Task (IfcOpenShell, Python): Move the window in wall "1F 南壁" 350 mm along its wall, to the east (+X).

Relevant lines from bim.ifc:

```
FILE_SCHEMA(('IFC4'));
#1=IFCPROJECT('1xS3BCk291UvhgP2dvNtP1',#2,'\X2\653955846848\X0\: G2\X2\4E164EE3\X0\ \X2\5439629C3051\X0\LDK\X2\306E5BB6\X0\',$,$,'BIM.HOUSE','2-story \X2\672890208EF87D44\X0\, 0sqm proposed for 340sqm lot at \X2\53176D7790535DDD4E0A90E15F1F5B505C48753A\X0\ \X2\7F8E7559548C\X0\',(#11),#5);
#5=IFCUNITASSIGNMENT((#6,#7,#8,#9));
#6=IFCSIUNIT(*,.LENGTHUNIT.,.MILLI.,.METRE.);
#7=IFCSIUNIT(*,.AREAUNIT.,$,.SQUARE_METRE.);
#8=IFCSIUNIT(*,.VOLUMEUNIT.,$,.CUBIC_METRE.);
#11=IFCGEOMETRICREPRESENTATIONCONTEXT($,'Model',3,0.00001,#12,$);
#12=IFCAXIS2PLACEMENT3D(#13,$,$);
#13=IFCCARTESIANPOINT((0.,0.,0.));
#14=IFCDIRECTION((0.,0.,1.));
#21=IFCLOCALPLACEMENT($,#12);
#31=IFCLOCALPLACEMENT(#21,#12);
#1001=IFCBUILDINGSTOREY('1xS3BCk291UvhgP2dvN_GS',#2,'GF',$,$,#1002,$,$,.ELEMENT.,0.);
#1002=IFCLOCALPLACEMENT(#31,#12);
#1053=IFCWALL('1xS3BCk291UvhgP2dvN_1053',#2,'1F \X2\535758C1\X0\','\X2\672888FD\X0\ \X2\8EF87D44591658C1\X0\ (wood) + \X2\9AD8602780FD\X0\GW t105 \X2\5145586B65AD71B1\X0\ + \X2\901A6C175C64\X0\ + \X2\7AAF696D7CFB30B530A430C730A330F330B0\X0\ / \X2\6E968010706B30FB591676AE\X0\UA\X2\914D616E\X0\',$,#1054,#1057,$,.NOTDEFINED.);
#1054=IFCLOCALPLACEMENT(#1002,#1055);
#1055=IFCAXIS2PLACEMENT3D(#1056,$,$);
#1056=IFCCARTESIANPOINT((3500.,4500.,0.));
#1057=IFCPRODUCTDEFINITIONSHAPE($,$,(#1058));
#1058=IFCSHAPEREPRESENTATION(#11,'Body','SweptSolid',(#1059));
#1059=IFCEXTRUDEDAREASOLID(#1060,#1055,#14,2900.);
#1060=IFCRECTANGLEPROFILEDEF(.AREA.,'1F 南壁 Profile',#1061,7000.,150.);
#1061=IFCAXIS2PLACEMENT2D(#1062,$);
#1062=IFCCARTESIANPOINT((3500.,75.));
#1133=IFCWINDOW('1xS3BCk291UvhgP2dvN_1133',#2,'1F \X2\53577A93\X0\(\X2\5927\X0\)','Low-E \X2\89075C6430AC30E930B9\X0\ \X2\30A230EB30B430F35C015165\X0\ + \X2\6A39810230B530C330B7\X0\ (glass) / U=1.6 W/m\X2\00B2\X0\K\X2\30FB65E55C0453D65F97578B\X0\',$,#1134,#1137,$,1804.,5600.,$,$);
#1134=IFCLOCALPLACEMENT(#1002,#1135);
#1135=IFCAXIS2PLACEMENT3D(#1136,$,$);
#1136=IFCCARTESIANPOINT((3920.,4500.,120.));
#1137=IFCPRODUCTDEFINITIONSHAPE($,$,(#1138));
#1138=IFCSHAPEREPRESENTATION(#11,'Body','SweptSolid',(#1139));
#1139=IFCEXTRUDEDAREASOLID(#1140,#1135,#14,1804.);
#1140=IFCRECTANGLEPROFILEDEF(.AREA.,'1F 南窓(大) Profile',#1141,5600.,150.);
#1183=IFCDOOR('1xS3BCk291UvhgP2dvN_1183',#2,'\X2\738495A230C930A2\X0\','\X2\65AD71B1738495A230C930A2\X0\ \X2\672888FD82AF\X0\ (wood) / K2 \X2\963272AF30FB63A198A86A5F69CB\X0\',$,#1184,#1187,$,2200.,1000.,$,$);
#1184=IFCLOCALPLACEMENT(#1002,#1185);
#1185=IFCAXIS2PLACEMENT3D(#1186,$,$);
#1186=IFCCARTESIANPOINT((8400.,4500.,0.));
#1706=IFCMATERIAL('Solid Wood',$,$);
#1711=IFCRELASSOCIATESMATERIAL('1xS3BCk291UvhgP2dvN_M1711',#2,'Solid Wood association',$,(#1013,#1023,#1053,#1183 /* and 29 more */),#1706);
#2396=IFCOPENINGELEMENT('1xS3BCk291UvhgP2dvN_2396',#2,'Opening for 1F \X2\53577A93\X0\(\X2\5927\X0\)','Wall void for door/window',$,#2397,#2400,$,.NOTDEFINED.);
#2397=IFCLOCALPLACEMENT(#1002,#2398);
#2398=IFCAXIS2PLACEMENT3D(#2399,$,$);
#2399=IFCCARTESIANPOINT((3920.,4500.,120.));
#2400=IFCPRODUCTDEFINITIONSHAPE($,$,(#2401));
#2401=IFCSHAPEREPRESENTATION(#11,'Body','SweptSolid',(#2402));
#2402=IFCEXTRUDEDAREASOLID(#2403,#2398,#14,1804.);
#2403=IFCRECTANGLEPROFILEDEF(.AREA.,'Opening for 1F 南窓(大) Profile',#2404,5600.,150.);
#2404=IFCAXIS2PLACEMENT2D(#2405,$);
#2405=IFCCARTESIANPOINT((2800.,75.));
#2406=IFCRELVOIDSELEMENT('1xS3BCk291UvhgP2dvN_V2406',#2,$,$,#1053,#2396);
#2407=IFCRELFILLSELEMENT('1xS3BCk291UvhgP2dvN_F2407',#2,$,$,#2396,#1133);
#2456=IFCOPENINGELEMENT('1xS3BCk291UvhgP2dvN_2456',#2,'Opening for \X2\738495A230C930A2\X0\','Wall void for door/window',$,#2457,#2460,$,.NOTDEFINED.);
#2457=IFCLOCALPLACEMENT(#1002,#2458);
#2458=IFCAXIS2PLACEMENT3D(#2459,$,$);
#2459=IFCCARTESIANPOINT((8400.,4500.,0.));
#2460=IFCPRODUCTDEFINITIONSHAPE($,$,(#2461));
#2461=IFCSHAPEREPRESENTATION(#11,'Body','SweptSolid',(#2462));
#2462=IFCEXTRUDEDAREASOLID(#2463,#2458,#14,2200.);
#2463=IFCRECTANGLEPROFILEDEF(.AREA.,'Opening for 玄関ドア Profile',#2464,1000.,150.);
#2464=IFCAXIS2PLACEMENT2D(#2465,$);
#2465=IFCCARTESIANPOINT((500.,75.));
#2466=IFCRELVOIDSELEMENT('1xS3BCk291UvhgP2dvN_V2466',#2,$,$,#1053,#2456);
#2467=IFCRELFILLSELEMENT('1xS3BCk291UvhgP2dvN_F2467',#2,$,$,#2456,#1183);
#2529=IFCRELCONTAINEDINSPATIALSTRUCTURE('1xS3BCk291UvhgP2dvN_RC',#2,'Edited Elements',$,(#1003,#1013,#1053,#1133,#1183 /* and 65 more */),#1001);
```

```python
import ifcopenshell
import ifcopenshell.api.geometry
import ifcopenshell.util.placement
import ifcopenshell.util.unit

model = ifcopenshell.open("bim.ifc")
unit_scale = ifcopenshell.util.unit.calculate_unit_scale(model)

window = model.by_guid("1xS3BCk291UvhgP2dvN_1133")
opening = window.FillsVoids[0].RelatingOpeningElement
wall = opening.VoidsElements[0].RelatingBuildingElement

wall_matrix = ifcopenshell.util.placement.get_local_placement(wall.ObjectPlacement)
shift = wall_matrix[:3, 0] * 0.35 / unit_scale
before = ifcopenshell.util.placement.get_local_placement(window.ObjectPlacement)[:3, 3].copy()

# The window is not placed relative to its opening, so move both.
for product in (opening, window):
    matrix = ifcopenshell.util.placement.get_local_placement(product.ObjectPlacement)
    matrix[:3, 3] += shift
    ifcopenshell.api.geometry.edit_object_placement(model, product=product, matrix=matrix, is_si=False)

after = ifcopenshell.util.placement.get_local_placement(window.ObjectPlacement)[:3, 3]
print("window moved by", (after - before).round(3) + 0.0)

model.write("bim_edited.ifc")
```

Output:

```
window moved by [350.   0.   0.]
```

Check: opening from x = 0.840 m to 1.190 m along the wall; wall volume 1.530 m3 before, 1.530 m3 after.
